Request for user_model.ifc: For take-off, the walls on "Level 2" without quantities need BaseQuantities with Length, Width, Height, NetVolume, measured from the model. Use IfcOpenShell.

First a look at what the model holds.

```python
import ifcopenshell
import ifcopenshell.util.element
import ifcopenshell.util.unit

model = ifcopenshell.open("user_model.ifc")
print(model.schema)
for unit_type in ("LENGTHUNIT", "AREAUNIT", "VOLUMEUNIT"):
    print(unit_type, ifcopenshell.util.unit.calculate_unit_scale(model, unit_type))
storey = next(s for s in model.by_type("IfcBuildingStorey") if s.Name == "Level 2")
walls = [e for e in ifcopenshell.util.element.get_decomposition(storey) if e.is_a("IfcWall")]
for e in sorted(walls, key=lambda e: e.id()):
    print(e.id(), e.is_a(), e.Name, list(ifcopenshell.util.element.get_psets(e, qtos_only=True)), sep=" | ")
```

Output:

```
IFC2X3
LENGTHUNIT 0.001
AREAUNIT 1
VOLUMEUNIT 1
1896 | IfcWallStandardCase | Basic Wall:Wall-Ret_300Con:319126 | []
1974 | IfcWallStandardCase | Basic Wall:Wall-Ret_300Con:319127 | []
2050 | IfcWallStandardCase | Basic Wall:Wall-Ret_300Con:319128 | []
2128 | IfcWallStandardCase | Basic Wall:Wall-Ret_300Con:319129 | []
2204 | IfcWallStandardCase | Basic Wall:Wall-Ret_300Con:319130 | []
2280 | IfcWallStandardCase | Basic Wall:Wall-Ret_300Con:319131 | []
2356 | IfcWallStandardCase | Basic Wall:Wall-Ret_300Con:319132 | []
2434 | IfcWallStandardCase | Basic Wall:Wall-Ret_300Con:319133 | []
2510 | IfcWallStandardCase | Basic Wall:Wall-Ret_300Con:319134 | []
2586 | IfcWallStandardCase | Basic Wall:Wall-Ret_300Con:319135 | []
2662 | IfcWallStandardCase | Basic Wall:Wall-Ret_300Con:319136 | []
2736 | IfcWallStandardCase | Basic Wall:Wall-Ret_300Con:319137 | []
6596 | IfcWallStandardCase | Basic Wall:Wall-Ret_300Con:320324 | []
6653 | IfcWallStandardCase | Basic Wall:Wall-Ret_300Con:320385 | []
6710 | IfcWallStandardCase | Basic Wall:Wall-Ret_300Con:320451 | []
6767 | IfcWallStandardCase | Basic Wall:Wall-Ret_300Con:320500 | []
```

```python
import ifcopenshell
import ifcopenshell.api.pset
import ifcopenshell.geom
import ifcopenshell.util.element
import ifcopenshell.util.shape
import ifcopenshell.util.unit

model = ifcopenshell.open("user_model.ifc")
unit_scale = ifcopenshell.util.unit.calculate_unit_scale(model)
volume_scale = ifcopenshell.util.unit.calculate_unit_scale(model, "VOLUMEUNIT")
settings = ifcopenshell.geom.settings()

storey = next(s for s in model.by_type("IfcBuildingStorey") if s.Name == "Level 2")
walls = [e for e in ifcopenshell.util.element.get_decomposition(storey) if e.is_a("IfcWall")]

for e in sorted(walls, key=lambda e: e.id()):
    if ifcopenshell.util.element.get_psets(e, qtos_only=True, should_inherit=False):
        continue
    # Geometry comes back in metres, in the element's own axes.
    shape = ifcopenshell.geom.create_shape(settings, e)
    values = {
        "Length": ifcopenshell.util.shape.get_x(shape.geometry) / unit_scale,
        "Width": ifcopenshell.util.shape.get_y(shape.geometry) / unit_scale,
        "Height": ifcopenshell.util.shape.get_z(shape.geometry) / unit_scale,
        "NetVolume": ifcopenshell.util.shape.get_volume(shape.geometry) / volume_scale,
    }
    qto = ifcopenshell.api.pset.add_qto(model, product=e, name="BaseQuantities")
    ifcopenshell.api.pset.edit_qto(model, qto=qto, properties=values)
    print(e.id(), {k: round(v, 3) for k, v in values.items()})

model.write("user_model_v2.ifc")
```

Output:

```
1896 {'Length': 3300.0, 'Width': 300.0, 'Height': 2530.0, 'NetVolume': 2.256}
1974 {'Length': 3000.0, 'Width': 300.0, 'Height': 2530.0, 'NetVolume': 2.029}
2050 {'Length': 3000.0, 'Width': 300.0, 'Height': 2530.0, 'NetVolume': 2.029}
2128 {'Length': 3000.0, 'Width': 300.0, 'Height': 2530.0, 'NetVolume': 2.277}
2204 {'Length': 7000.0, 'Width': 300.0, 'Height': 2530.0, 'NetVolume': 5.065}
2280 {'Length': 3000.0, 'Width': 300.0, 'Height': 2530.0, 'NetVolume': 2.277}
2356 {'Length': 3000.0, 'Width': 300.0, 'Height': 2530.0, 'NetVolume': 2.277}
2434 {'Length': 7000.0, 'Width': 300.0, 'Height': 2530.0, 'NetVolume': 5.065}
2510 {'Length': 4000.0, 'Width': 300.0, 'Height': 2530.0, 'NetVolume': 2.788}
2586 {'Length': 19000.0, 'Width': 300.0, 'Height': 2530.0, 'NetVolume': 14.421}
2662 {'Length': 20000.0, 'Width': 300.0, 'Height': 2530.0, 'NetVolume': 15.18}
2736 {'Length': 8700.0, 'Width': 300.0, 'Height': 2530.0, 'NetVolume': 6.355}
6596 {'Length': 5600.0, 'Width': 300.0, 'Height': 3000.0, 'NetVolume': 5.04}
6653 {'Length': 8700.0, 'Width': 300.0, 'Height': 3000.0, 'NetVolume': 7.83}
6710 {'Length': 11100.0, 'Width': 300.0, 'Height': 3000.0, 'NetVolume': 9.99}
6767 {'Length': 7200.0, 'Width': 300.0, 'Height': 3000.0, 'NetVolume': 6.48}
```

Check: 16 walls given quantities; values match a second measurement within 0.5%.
